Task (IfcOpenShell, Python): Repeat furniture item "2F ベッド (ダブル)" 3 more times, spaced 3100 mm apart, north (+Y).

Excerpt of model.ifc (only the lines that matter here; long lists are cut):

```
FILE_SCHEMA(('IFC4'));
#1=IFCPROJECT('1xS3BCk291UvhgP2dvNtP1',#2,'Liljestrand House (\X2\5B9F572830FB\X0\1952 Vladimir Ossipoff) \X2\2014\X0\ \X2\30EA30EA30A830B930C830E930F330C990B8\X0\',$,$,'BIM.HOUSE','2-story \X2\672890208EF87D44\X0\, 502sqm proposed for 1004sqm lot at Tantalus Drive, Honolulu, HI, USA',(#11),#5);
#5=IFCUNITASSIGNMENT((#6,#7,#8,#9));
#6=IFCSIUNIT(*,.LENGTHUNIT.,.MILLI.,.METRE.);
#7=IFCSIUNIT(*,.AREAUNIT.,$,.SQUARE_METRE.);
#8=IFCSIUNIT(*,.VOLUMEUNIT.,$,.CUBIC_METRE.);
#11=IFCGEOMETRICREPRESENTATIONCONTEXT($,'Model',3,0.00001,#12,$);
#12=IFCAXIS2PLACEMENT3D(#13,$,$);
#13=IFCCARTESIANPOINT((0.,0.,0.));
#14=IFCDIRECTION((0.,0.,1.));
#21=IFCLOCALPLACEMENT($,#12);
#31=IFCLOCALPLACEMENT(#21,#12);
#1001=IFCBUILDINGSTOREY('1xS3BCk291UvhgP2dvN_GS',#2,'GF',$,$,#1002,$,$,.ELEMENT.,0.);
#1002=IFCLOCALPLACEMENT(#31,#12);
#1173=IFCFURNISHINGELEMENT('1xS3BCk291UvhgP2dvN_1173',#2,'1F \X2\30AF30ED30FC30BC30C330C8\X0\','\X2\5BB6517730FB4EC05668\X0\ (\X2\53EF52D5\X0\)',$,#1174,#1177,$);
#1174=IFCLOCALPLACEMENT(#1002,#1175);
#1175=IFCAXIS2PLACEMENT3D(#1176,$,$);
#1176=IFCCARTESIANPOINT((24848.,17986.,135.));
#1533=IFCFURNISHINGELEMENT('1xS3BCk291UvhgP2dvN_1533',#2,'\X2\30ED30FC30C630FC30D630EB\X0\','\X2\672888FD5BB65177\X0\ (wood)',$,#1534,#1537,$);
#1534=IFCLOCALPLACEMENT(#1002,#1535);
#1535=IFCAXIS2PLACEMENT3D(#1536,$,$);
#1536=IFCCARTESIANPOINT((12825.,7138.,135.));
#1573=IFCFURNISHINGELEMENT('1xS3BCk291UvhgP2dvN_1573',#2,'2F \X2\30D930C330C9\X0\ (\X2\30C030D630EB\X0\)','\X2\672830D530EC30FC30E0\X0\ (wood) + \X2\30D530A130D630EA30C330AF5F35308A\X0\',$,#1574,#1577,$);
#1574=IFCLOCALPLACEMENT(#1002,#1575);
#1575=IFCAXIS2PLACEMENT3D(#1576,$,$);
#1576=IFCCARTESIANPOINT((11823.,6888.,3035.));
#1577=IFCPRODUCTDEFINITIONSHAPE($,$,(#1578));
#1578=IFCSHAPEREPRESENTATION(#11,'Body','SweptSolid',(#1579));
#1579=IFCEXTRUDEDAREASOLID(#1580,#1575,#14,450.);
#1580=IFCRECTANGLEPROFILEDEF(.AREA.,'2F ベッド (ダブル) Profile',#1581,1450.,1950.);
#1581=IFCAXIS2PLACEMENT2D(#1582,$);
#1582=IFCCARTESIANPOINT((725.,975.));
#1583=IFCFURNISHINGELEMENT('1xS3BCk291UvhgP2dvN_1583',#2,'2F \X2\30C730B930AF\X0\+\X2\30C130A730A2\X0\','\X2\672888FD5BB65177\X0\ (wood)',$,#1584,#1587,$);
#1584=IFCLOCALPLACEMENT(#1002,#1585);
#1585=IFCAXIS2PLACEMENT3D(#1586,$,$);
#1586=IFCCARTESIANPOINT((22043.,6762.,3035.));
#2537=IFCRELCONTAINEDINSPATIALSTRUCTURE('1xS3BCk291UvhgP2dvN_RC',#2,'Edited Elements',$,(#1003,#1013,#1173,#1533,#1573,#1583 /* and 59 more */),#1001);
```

```python
import numpy as np
import ifcopenshell
import ifcopenshell.api.geometry
import ifcopenshell.api.root
import ifcopenshell.util.element
import ifcopenshell.util.placement

model = ifcopenshell.open("model.ifc")


def reuse_history(source, copy):
    """copy_class also copies each property set's owner history, people and application; keep the originals."""
    for rel in copy.IsDefinedBy:
        if rel.is_a("IfcRelDefinesByProperties") and (history := rel.RelatingPropertyDefinition.OwnerHistory):
            rel.RelatingPropertyDefinition.OwnerHistory = source.OwnerHistory
            ifcopenshell.util.element.remove_deep2(model, history)


source = model.by_guid("1xS3BCk291UvhgP2dvN_1573")
base = ifcopenshell.util.placement.get_local_placement(source.ObjectPlacement)
step = np.array([0.0, 1.0, 0.0]) * 3100.0

for i in range(1, 4):
    copy = ifcopenshell.api.root.copy_class(model, product=source)
    copy.Representation = ifcopenshell.util.element.copy_deep(
        model, source.Representation, exclude=["IfcGeometricRepresentationContext", "IfcRepresentationMap"]
    )
    reuse_history(source, copy)
    matrix = base.copy()
    matrix[:3, 3] += i * step
    print("added at", matrix[:3, 3].round(3) + 0.0)
    ifcopenshell.api.geometry.edit_object_placement(model, product=copy, matrix=matrix, is_si=False)

model.write("model_edited.ifc")
```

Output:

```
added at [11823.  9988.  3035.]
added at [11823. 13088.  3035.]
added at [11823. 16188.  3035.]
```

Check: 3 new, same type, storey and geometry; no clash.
